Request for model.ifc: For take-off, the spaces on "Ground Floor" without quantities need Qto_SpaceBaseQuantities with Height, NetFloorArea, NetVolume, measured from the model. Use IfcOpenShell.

First a look at what the model holds.

```python
import ifcopenshell
import ifcopenshell.util.element
import ifcopenshell.util.unit

model = ifcopenshell.open("model.ifc")
print(model.schema)
for unit_type in ("LENGTHUNIT", "AREAUNIT", "VOLUMEUNIT"):
    print(unit_type, ifcopenshell.util.unit.calculate_unit_scale(model, unit_type))
storey = next(s for s in model.by_type("IfcBuildingStorey") if s.Name == "Ground Floor")
spaces = [e for e in ifcopenshell.util.element.get_decomposition(storey) if e.is_a("IfcSpace")]
for e in sorted(spaces, key=lambda e: e.id()):
    print(e.id(), e.is_a(), e.Name, list(ifcopenshell.util.element.get_psets(e, qtos_only=True)), sep=" | ")
```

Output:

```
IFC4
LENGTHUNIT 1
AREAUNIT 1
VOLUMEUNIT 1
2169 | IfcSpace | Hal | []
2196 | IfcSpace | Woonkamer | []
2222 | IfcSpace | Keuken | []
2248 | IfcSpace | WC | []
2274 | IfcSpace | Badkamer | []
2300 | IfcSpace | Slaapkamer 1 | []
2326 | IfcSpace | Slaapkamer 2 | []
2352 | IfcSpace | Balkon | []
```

```python
import ifcopenshell
import ifcopenshell.api.pset
import ifcopenshell.geom
import ifcopenshell.util.element
import ifcopenshell.util.shape
import ifcopenshell.util.unit

model = ifcopenshell.open("model.ifc")
unit_scale = ifcopenshell.util.unit.calculate_unit_scale(model)
area_scale = ifcopenshell.util.unit.calculate_unit_scale(model, "AREAUNIT")
volume_scale = ifcopenshell.util.unit.calculate_unit_scale(model, "VOLUMEUNIT")
settings = ifcopenshell.geom.settings()

storey = next(s for s in model.by_type("IfcBuildingStorey") if s.Name == "Ground Floor")
spaces = [e for e in ifcopenshell.util.element.get_decomposition(storey) if e.is_a("IfcSpace")]

for e in sorted(spaces, key=lambda e: e.id()):
    if ifcopenshell.util.element.get_psets(e, qtos_only=True, should_inherit=False):
        continue
    # Geometry comes back in metres, in the element's own axes.
    shape = ifcopenshell.geom.create_shape(settings, e)
    values = {
        "Height": ifcopenshell.util.shape.get_z(shape.geometry) / unit_scale,
        "NetFloorArea": ifcopenshell.util.shape.get_footprint_area(shape.geometry) / area_scale,
        "NetVolume": ifcopenshell.util.shape.get_volume(shape.geometry) / volume_scale,
    }
    qto = ifcopenshell.api.pset.add_qto(model, product=e, name="Qto_SpaceBaseQuantities")
    ifcopenshell.api.pset.edit_qto(model, qto=qto, properties=values)
    print(e.id(), {k: round(v, 3) for k, v in values.items()})

model.write("model_edited.ifc")
```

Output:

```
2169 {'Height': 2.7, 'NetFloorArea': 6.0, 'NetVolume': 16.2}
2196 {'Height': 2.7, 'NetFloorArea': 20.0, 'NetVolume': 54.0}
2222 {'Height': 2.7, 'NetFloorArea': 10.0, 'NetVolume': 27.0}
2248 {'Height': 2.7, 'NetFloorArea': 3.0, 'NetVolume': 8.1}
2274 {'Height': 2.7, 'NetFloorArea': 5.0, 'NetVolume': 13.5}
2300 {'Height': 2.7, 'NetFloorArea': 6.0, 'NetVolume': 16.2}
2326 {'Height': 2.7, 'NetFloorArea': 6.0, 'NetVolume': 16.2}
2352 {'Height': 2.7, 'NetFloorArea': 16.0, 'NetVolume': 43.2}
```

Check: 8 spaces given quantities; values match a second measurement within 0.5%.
